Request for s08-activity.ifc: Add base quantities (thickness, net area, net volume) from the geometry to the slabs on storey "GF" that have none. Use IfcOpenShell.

First a look at what the model holds.

```python
import ifcopenshell
import ifcopenshell.util.element
import ifcopenshell.util.unit

model = ifcopenshell.open("s08-activity.ifc")
print(model.schema)
for unit_type in ("LENGTHUNIT", "AREAUNIT", "VOLUMEUNIT"):
    print(unit_type, ifcopenshell.util.unit.calculate_unit_scale(model, unit_type))
storey = next(s for s in model.by_type("IfcBuildingStorey") if s.Name == "GF")
slabs = [e for e in ifcopenshell.util.element.get_decomposition(storey) if e.is_a("IfcSlab")]
for e in sorted(slabs, key=lambda e: e.id()):
    print(e.id(), e.is_a(), e.Name, list(ifcopenshell.util.element.get_psets(e, qtos_only=True)), sep=" | ")
```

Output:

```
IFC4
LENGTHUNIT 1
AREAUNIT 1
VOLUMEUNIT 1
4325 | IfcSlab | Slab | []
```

```python
import ifcopenshell
import ifcopenshell.api.pset
import ifcopenshell.geom
import ifcopenshell.util.element
import ifcopenshell.util.shape
import ifcopenshell.util.unit

model = ifcopenshell.open("s08-activity.ifc")
unit_scale = ifcopenshell.util.unit.calculate_unit_scale(model)
area_scale = ifcopenshell.util.unit.calculate_unit_scale(model, "AREAUNIT")
volume_scale = ifcopenshell.util.unit.calculate_unit_scale(model, "VOLUMEUNIT")
settings = ifcopenshell.geom.settings()

storey = next(s for s in model.by_type("IfcBuildingStorey") if s.Name == "GF")
slabs = [e for e in ifcopenshell.util.element.get_decomposition(storey) if e.is_a("IfcSlab")]

for e in sorted(slabs, key=lambda e: e.id()):
    if ifcopenshell.util.element.get_psets(e, qtos_only=True, should_inherit=False):
        continue
    # Geometry comes back in metres, in the element's own axes.
    shape = ifcopenshell.geom.create_shape(settings, e)
    values = {
        "Width": ifcopenshell.util.shape.get_z(shape.geometry) / unit_scale,
        "NetArea": ifcopenshell.util.shape.get_footprint_area(shape.geometry) / area_scale,
        "NetVolume": ifcopenshell.util.shape.get_volume(shape.geometry) / volume_scale,
    }
    qto = ifcopenshell.api.pset.add_qto(model, product=e, name="Qto_SlabBaseQuantities")
    ifcopenshell.api.pset.edit_qto(model, qto=qto, properties=values)
    print(e.id(), {k: round(v, 3) for k, v in values.items()})

model.write("s08-activity_rev.ifc")
```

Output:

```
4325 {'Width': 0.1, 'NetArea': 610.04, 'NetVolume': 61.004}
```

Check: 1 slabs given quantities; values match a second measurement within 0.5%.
